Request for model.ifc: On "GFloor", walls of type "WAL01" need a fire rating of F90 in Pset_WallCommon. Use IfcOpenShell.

First a look at what the model holds.

```python
import ifcopenshell
import ifcopenshell.util.element

model = ifcopenshell.open("model.ifc")
print(model.schema)
storey = next(s for s in model.by_type("IfcBuildingStorey") if s.Name == "GFloor")
walls = [e for e in ifcopenshell.util.element.get_decomposition(storey) if e.is_a("IfcWall")]
seen = {}
for e in walls:
    element_type = ifcopenshell.util.element.get_type(e)
    key = (element_type.Name if element_type != e and element_type else None, ifcopenshell.util.element.get_pset(e, "Pset_WallCommon", "FireRating"))
    seen[key] = seen.get(key, 0) + 1
for (name, value), count in sorted(seen.items(), key=str):
    print(count, "x", name, "|", value)
```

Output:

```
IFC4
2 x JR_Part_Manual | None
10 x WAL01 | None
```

```python
import ifcopenshell
import ifcopenshell.api.pset
import ifcopenshell.util.element

model = ifcopenshell.open("model.ifc")

storey = next(s for s in model.by_type("IfcBuildingStorey") if s.Name == "GFloor")
walls = [e for e in ifcopenshell.util.element.get_decomposition(storey) if e.is_a("IfcWall")]

count = 0
for e in walls:
    element_type = ifcopenshell.util.element.get_type(e)
    if element_type in (None, e) or element_type.Name != "WAL01":
        continue
    # add_pset returns the element's existing set when there is one.
    pset = ifcopenshell.api.pset.add_pset(model, product=e, name="Pset_WallCommon")
    ifcopenshell.api.pset.edit_pset(model, pset=pset, properties={"FireRating": "F90"})
    count += 1

print(count, "walls updated")

model.write("model-out.ifc")
```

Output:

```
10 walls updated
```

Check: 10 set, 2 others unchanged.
